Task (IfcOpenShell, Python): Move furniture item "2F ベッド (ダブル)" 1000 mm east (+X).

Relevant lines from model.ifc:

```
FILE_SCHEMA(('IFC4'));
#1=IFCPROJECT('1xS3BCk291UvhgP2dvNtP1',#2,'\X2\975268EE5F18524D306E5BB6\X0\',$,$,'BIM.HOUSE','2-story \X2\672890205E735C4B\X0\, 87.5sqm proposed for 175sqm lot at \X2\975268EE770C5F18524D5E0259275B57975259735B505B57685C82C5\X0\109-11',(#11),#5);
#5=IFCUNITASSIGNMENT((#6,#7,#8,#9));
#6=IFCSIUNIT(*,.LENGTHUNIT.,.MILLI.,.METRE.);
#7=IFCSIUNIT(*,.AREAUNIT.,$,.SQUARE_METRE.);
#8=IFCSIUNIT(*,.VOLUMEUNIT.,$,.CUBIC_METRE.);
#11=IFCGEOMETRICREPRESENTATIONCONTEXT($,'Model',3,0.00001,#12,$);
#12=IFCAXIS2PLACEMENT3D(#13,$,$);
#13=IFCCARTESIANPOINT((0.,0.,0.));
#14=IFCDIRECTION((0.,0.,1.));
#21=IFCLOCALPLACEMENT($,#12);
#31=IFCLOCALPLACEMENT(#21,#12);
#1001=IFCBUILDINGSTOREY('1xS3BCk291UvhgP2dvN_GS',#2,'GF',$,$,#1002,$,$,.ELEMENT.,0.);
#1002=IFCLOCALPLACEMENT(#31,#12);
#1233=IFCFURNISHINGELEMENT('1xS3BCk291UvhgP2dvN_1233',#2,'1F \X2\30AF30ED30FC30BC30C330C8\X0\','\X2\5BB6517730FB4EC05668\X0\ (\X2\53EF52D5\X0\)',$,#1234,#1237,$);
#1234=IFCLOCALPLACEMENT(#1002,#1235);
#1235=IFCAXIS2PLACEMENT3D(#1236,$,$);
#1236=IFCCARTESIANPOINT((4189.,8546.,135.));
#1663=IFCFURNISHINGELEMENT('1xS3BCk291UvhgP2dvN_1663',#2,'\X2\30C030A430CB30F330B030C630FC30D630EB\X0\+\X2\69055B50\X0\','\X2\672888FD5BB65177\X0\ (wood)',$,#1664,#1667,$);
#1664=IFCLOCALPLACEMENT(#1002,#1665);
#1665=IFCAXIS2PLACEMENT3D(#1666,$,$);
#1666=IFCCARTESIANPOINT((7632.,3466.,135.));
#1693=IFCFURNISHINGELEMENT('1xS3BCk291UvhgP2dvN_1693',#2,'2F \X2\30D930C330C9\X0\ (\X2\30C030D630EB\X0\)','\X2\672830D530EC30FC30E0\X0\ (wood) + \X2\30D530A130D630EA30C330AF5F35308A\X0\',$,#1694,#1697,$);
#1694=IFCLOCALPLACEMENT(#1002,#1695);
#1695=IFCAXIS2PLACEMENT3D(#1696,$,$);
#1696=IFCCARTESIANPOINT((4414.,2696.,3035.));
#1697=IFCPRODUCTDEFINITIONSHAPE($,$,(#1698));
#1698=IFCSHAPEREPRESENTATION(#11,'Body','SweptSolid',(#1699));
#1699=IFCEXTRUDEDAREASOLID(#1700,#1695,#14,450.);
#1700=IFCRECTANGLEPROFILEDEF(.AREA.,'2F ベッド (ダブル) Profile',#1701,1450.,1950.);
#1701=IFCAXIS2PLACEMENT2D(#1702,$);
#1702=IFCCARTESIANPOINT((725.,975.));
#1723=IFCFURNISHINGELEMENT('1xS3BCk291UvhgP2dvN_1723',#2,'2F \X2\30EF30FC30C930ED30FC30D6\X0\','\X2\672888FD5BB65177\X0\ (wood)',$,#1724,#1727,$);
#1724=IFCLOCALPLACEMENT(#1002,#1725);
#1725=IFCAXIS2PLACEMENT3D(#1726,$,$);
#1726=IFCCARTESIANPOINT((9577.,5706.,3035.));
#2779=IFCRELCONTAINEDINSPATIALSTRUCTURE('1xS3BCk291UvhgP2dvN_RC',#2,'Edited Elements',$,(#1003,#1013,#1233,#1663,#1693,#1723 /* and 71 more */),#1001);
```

```python
import ifcopenshell
import ifcopenshell.api.geometry
import ifcopenshell.util.placement
import ifcopenshell.util.unit

model = ifcopenshell.open("model.ifc")
unit_scale = ifcopenshell.util.unit.calculate_unit_scale(model)

item = model.by_id(1693)
matrix = ifcopenshell.util.placement.get_local_placement(item.ObjectPlacement)
matrix[0, 3] += 1 / unit_scale
ifcopenshell.api.geometry.edit_object_placement(model, product=item, matrix=matrix, is_si=False)

print(ifcopenshell.util.placement.get_local_placement(item.ObjectPlacement).round(3) + 0.0)

model.write("model-out.ifc")
```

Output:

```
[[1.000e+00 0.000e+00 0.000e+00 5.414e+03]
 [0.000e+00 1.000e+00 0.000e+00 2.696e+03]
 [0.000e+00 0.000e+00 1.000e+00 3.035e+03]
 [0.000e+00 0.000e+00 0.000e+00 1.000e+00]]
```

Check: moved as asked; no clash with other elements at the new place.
